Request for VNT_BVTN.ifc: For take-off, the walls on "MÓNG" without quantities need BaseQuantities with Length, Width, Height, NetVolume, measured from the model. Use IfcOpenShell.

First a look at what the model holds.

```python
import ifcopenshell
import ifcopenshell.util.element
import ifcopenshell.util.unit

model = ifcopenshell.open("VNT_BVTN.ifc")
print(model.schema)
for unit_type in ("LENGTHUNIT", "AREAUNIT", "VOLUMEUNIT"):
    print(unit_type, ifcopenshell.util.unit.calculate_unit_scale(model, unit_type))
storey = next(s for s in model.by_type("IfcBuildingStorey") if s.Name == "MÓNG")
walls = [e for e in ifcopenshell.util.element.get_decomposition(storey) if e.is_a("IfcWall")]
for e in sorted(walls, key=lambda e: e.id()):
    print(e.id(), e.is_a(), e.Name, list(ifcopenshell.util.element.get_psets(e, qtos_only=True)), sep=" | ")
```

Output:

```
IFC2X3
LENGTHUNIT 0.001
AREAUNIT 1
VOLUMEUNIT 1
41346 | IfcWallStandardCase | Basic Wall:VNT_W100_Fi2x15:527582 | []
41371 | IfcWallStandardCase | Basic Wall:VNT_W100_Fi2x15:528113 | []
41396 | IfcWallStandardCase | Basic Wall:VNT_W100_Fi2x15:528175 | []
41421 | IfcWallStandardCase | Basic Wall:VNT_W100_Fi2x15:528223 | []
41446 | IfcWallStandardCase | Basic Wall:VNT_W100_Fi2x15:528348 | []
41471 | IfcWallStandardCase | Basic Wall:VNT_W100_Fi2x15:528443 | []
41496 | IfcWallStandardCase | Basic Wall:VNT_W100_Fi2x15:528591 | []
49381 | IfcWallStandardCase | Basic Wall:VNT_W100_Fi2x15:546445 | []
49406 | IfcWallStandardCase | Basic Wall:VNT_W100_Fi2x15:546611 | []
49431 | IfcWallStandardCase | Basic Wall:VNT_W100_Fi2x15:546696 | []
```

```python
import ifcopenshell
import ifcopenshell.api.pset
import ifcopenshell.geom
import ifcopenshell.util.element
import ifcopenshell.util.shape
import ifcopenshell.util.unit

model = ifcopenshell.open("VNT_BVTN.ifc")
unit_scale = ifcopenshell.util.unit.calculate_unit_scale(model)
volume_scale = ifcopenshell.util.unit.calculate_unit_scale(model, "VOLUMEUNIT")
settings = ifcopenshell.geom.settings()

storey = next(s for s in model.by_type("IfcBuildingStorey") if s.Name == "MÓNG")
walls = [e for e in ifcopenshell.util.element.get_decomposition(storey) if e.is_a("IfcWall")]

for e in sorted(walls, key=lambda e: e.id()):
    if ifcopenshell.util.element.get_psets(e, qtos_only=True, should_inherit=False):
        continue
    # Geometry comes back in metres, in the element's own axes.
    shape = ifcopenshell.geom.create_shape(settings, e)
    values = {
        "Length": ifcopenshell.util.shape.get_x(shape.geometry) / unit_scale,
        "Width": ifcopenshell.util.shape.get_y(shape.geometry) / unit_scale,
        "Height": ifcopenshell.util.shape.get_z(shape.geometry) / unit_scale,
        "NetVolume": ifcopenshell.util.shape.get_volume(shape.geometry) / volume_scale,
    }
    qto = ifcopenshell.api.pset.add_qto(model, product=e, name="BaseQuantities")
    ifcopenshell.api.pset.edit_qto(model, qto=qto, properties=values)
    print(e.id(), {k: round(v, 3) for k, v in values.items()})

model.write("VNT_BVTN-out.ifc")
```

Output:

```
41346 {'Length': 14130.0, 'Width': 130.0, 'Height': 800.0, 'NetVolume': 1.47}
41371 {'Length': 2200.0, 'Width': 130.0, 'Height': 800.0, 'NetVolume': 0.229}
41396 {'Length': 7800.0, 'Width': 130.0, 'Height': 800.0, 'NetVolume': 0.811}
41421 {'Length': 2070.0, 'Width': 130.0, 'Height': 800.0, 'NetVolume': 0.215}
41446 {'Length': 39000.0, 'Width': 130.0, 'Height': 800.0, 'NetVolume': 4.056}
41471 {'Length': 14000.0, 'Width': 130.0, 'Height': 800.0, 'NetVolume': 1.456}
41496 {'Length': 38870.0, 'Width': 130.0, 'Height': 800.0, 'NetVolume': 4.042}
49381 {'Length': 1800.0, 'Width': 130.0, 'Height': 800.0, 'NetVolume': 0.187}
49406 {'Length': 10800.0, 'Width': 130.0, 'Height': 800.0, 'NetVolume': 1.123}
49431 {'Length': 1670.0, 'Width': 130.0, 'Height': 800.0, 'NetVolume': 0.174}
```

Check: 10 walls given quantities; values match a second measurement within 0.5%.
